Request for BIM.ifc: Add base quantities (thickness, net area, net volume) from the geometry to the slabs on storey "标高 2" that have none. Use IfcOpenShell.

First a look at what the model holds.

```python
import ifcopenshell
import ifcopenshell.util.element
import ifcopenshell.util.unit

model = ifcopenshell.open("BIM.ifc")
print(model.schema)
for unit_type in ("LENGTHUNIT", "AREAUNIT", "VOLUMEUNIT"):
    print(unit_type, ifcopenshell.util.unit.calculate_unit_scale(model, unit_type))
storey = next(s for s in model.by_type("IfcBuildingStorey") if s.Name == "标高 2")
slabs = [e for e in ifcopenshell.util.element.get_decomposition(storey) if e.is_a("IfcSlab")]
for e in sorted(slabs, key=lambda e: e.id()):
    print(e.id(), e.is_a(), e.Name, list(ifcopenshell.util.element.get_psets(e, qtos_only=True)), sep=" | ")
```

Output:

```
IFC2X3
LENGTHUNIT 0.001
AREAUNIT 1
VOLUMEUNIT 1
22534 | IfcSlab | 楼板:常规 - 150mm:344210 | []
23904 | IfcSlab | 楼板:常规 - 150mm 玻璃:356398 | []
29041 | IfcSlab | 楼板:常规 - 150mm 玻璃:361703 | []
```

```python
import ifcopenshell
import ifcopenshell.api.pset
import ifcopenshell.geom
import ifcopenshell.util.element
import ifcopenshell.util.shape
import ifcopenshell.util.unit

model = ifcopenshell.open("BIM.ifc")
unit_scale = ifcopenshell.util.unit.calculate_unit_scale(model)
area_scale = ifcopenshell.util.unit.calculate_unit_scale(model, "AREAUNIT")
volume_scale = ifcopenshell.util.unit.calculate_unit_scale(model, "VOLUMEUNIT")
settings = ifcopenshell.geom.settings()

storey = next(s for s in model.by_type("IfcBuildingStorey") if s.Name == "标高 2")
slabs = [e for e in ifcopenshell.util.element.get_decomposition(storey) if e.is_a("IfcSlab")]

for e in sorted(slabs, key=lambda e: e.id()):
    if ifcopenshell.util.element.get_psets(e, qtos_only=True, should_inherit=False):
        continue
    # Geometry comes back in metres, in the element's own axes.
    shape = ifcopenshell.geom.create_shape(settings, e)
    values = {
        "Width": ifcopenshell.util.shape.get_z(shape.geometry) / unit_scale,
        "NetArea": ifcopenshell.util.shape.get_footprint_area(shape.geometry) / area_scale,
        "NetVolume": ifcopenshell.util.shape.get_volume(shape.geometry) / volume_scale,
    }
    qto = ifcopenshell.api.pset.add_qto(model, product=e, name="BaseQuantities")
    ifcopenshell.api.pset.edit_qto(model, qto=qto, properties=values)
    print(e.id(), {k: round(v, 3) for k, v in values.items()})

model.write("BIM_updated.ifc")
```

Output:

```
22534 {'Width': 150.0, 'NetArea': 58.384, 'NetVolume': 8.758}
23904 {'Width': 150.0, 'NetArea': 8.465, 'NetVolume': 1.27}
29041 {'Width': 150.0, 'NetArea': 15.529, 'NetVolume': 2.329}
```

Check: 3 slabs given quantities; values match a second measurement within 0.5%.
